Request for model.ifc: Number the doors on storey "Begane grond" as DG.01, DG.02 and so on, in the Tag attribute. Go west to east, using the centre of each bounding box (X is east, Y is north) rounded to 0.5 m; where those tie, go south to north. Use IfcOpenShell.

First a look at what the model holds.

```python
import ifcopenshell
import ifcopenshell.util.element
import ifcopenshell.util.placement

model = ifcopenshell.open("model.ifc")
print(model.schema)
storey = next(s for s in model.by_type("IfcBuildingStorey") if s.Name == "Begane grond")
doors = [e for e in ifcopenshell.util.element.get_decomposition(storey) if e.is_a("IfcDoor")]
for e in sorted(doors, key=lambda e: e.id()):
    origin = ifcopenshell.util.placement.get_local_placement(e.ObjectPlacement)[:3, 3]
    print(e.id(), e.Tag, e.Name, origin.round(2) + 0.0, sep=" | ")
```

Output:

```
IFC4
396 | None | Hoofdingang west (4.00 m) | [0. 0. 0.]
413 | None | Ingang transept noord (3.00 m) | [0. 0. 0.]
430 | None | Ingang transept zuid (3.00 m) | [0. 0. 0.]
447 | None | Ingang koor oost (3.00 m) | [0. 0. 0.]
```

```python
import ifcopenshell
import ifcopenshell.geom
import ifcopenshell.util.element
import ifcopenshell.util.shape

model = ifcopenshell.open("model.ifc")
settings = ifcopenshell.geom.settings()
settings.set("use-world-coords", True)


def centre(element):
    shape = ifcopenshell.geom.create_shape(settings, element)
    return ifcopenshell.util.shape.get_bbox_centroid(shape.geometry)


storey = next(s for s in model.by_type("IfcBuildingStorey") if s.Name == "Begane grond")
doors = [e for e in ifcopenshell.util.element.get_decomposition(storey) if e.is_a("IfcDoor")]

# Insertion points can sit at a corner or the storey origin, so sort by the geometry (in metres).
centres = {e: centre(e) for e in doors}
doors.sort(key=lambda e: (round(centres[e][0] / 0.5), centres[e][1]))

for i, e in enumerate(doors, start=1):
    number = f"DG.{i:02d}"
    e.Tag = number
    print(e.id(), number)

model.write("model_rev.ifc")
```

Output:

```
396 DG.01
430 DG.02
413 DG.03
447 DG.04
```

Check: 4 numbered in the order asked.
